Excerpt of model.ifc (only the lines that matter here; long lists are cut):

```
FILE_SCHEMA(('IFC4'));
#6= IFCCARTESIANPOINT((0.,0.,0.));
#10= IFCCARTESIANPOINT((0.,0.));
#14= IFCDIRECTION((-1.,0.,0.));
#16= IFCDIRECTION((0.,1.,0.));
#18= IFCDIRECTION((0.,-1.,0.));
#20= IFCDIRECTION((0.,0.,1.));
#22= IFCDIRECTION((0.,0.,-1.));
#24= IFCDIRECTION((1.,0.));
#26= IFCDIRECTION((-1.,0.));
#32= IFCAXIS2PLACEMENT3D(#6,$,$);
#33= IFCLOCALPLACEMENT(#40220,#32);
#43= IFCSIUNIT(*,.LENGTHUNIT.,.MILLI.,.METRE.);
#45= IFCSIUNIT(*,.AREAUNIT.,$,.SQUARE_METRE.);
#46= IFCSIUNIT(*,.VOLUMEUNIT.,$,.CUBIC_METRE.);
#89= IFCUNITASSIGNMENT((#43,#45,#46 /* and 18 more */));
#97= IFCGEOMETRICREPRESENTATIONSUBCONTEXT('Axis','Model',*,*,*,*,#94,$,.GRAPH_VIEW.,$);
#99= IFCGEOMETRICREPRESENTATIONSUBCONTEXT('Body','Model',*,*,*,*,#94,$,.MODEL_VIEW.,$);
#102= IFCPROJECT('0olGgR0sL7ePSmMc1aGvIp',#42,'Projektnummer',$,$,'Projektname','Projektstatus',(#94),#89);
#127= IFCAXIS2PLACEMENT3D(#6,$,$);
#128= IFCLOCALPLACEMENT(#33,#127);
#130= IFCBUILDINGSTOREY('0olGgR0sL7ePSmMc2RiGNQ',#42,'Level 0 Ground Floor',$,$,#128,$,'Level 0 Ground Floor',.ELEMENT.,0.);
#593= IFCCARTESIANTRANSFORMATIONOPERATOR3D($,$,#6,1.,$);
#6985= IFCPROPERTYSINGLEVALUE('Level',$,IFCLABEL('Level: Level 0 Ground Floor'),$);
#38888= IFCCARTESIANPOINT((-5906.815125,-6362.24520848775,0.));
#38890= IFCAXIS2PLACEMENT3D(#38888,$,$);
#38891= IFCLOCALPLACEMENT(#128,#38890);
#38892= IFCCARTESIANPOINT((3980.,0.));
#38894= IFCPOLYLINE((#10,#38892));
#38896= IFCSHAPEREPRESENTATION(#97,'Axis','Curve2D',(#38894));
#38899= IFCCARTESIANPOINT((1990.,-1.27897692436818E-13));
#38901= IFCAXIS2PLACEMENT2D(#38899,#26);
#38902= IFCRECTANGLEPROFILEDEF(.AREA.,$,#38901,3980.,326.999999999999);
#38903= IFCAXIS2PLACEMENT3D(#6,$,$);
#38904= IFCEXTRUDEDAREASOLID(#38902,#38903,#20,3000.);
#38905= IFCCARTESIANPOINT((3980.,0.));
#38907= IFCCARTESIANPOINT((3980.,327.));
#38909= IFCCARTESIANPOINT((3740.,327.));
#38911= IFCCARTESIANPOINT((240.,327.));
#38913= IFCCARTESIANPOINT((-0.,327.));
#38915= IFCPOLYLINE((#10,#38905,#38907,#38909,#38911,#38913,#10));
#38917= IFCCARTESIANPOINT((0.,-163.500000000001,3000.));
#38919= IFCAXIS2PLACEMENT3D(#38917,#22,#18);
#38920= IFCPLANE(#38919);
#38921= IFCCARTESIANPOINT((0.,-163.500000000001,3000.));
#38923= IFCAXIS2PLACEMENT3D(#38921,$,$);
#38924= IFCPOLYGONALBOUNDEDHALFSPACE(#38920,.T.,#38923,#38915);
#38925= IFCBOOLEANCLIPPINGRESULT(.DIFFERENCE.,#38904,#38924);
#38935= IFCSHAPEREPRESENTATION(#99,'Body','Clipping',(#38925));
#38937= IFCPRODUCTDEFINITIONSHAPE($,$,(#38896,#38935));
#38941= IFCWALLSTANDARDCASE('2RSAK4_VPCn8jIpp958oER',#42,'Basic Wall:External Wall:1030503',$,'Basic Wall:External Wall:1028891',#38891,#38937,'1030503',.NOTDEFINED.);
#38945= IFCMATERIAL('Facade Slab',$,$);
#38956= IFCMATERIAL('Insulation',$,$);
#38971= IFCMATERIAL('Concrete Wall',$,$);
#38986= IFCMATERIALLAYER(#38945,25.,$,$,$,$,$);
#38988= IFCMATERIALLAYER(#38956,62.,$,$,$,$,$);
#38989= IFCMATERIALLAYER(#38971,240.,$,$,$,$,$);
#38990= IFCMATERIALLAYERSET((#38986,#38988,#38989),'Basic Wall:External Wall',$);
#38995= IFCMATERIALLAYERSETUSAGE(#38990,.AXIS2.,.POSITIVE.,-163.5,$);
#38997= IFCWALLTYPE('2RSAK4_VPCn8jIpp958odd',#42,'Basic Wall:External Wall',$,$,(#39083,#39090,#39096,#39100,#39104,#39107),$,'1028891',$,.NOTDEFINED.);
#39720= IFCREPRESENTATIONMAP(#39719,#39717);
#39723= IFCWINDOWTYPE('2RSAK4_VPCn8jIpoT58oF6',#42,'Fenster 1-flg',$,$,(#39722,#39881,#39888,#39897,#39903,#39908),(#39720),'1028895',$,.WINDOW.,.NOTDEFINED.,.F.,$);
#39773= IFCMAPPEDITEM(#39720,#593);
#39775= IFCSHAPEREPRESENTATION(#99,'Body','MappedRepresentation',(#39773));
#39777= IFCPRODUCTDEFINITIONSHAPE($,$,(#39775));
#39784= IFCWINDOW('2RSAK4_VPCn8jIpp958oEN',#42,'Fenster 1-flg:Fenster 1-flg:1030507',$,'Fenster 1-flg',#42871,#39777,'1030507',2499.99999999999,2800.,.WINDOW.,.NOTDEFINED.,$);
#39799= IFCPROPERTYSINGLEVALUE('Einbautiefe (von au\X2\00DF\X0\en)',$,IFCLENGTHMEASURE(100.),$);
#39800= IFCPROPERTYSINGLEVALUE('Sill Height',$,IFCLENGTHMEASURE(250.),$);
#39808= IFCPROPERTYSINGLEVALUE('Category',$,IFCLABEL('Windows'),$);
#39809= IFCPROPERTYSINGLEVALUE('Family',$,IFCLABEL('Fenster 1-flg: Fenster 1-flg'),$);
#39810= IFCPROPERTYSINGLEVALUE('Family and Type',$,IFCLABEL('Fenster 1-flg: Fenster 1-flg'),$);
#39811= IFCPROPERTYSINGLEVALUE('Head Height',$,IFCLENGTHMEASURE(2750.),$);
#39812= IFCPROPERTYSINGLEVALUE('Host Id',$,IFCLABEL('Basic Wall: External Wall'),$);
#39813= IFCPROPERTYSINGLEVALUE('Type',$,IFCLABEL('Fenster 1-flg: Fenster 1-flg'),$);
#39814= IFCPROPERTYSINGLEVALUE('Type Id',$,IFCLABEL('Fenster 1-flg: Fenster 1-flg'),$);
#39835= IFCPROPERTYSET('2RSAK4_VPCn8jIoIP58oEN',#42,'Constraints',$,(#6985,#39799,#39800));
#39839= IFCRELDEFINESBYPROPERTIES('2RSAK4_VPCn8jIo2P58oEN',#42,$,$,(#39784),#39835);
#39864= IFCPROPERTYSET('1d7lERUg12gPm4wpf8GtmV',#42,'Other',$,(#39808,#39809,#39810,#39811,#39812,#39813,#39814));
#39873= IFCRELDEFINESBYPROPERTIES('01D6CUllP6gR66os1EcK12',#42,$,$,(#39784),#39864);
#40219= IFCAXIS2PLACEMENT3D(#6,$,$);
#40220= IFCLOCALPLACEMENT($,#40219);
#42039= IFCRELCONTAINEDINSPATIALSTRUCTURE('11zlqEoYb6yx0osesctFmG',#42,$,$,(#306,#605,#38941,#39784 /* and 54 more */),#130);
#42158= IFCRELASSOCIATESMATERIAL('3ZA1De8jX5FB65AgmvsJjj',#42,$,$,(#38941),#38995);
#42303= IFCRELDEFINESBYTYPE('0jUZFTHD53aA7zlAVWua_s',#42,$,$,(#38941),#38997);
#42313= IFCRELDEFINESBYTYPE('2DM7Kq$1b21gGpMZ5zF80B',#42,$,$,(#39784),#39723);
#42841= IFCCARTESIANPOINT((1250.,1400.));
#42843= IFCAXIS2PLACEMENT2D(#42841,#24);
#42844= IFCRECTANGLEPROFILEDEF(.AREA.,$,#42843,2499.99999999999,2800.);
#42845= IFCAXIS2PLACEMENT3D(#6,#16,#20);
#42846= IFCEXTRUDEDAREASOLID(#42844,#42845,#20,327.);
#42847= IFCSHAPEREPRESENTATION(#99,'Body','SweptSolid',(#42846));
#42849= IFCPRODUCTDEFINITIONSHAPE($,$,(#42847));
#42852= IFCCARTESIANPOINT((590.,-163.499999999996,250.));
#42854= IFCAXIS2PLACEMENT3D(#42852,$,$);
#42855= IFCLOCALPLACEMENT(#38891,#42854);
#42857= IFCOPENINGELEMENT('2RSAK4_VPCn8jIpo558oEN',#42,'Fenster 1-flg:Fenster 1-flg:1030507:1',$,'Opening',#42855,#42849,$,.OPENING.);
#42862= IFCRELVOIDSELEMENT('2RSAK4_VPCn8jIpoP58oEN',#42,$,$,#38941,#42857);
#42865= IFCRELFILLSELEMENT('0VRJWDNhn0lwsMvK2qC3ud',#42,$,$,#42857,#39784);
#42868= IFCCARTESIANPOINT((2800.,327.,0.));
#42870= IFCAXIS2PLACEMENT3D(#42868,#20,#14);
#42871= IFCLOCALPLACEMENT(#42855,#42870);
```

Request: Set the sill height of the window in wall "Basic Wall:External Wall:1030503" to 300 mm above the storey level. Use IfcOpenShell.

```python
import numpy as np
import ifcopenshell
import ifcopenshell.api.geometry
import ifcopenshell.api.pset
import ifcopenshell.geom
import ifcopenshell.util.element
import ifcopenshell.util.placement
import ifcopenshell.util.shape
import ifcopenshell.util.unit

model = ifcopenshell.open("model.ifc")
unit_scale = ifcopenshell.util.unit.calculate_unit_scale(model)

window = model.by_guid("2RSAK4_VPCn8jIpp958oEN")
opening = window.FillsVoids[0].RelatingOpeningElement
storey = ifcopenshell.util.element.get_container(window, ifc_class="IfcBuildingStorey")
level = ifcopenshell.util.placement.get_local_placement(storey.ObjectPlacement)[2, 3]

# The opening's origin need not be at the sill, so measure its lowest point.
shape = ifcopenshell.geom.create_shape(ifcopenshell.geom.settings(), opening)
bottom = ifcopenshell.util.shape.get_shape_bottom_elevation(shape, shape.geometry) / unit_scale
dz = level + 0.3 / unit_scale - bottom

shift = np.array([0.0, 0.0, dz])
# The window is placed relative to its opening, so it follows when the opening moves.
matrix = ifcopenshell.util.placement.get_local_placement(opening.ObjectPlacement)
matrix[:3, 3] += shift
ifcopenshell.api.geometry.edit_object_placement(
    model, product=opening, matrix=matrix, is_si=False, should_transform_children=True
)

# Keep the stored heights in step.
pset = model.by_id(ifcopenshell.util.element.get_pset(window, "Constraints", should_inherit=False)["id"])
ifcopenshell.api.pset.edit_pset(model, pset=pset, properties={
    "Sill Height": model.create_entity("IfcLengthMeasure", ifcopenshell.util.element.get_pset(window, "Constraints", "Sill Height") + dz),
})
pset = model.by_id(ifcopenshell.util.element.get_pset(window, "Other", should_inherit=False)["id"])
ifcopenshell.api.pset.edit_pset(model, pset=pset, properties={
    "Head Height": model.create_entity("IfcLengthMeasure", ifcopenshell.util.element.get_pset(window, "Other", "Head Height") + dz),
})

print(f"moved by {dz * unit_scale:+.3f} m")

model.write("model-out.ifc")
```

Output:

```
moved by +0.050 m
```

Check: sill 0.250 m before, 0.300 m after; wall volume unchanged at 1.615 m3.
